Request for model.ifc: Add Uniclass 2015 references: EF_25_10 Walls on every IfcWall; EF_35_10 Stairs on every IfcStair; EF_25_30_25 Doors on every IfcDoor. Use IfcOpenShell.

First a look at what the model holds.

```python
import ifcopenshell

model = ifcopenshell.open("model.ifc")
print(model.schema)
print("classifications:", [c.Name for c in model.by_type("IfcClassification")])
for ifc_class in ("IfcDoor", "IfcRoof", "IfcStair", "IfcWall", "IfcWindow"):
    print(ifc_class, len(model.by_type(ifc_class)))
```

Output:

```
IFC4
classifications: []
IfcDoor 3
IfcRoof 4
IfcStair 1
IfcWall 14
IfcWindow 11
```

```python
import ifcopenshell
import ifcopenshell.api.classification

model = ifcopenshell.open("model.ifc")

system = ifcopenshell.api.classification.add_classification(model, classification="Uniclass 2015")

codes = {
    "IfcWall": ("EF_25_10", "Walls"),
    "IfcStair": ("EF_35_10", "Stairs"),
    "IfcDoor": ("EF_25_30_25", "Doors"),
}
for ifc_class, (code, name) in codes.items():
    products = model.by_type(ifc_class)
    ifcopenshell.api.classification.add_reference(
        model, products=products, classification=system, identification=code, name=name
    )
    print(code, len(products))

model.write("model_edited.ifc")
```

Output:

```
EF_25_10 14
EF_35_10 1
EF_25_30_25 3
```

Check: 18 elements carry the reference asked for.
